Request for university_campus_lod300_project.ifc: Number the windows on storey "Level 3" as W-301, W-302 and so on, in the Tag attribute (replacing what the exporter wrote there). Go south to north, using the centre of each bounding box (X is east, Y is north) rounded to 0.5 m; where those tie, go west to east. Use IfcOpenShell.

First a look at what the model holds.

```python
import ifcopenshell
import ifcopenshell.util.element
import ifcopenshell.util.placement

model = ifcopenshell.open("university_campus_lod300_project.ifc")
print(model.schema)
storey = next(s for s in model.by_type("IfcBuildingStorey") if s.Name == "Level 3")
windows = [e for e in ifcopenshell.util.element.get_decomposition(storey) if e.is_a("IfcWindow")]
for e in sorted(windows, key=lambda e: e.id()):
    origin = ifcopenshell.util.placement.get_local_placement(e.ObjectPlacement)[:3, 3]
    print(e.id(), e.Tag, e.Name, origin.round(2) + 0.0, sep=" | ")
```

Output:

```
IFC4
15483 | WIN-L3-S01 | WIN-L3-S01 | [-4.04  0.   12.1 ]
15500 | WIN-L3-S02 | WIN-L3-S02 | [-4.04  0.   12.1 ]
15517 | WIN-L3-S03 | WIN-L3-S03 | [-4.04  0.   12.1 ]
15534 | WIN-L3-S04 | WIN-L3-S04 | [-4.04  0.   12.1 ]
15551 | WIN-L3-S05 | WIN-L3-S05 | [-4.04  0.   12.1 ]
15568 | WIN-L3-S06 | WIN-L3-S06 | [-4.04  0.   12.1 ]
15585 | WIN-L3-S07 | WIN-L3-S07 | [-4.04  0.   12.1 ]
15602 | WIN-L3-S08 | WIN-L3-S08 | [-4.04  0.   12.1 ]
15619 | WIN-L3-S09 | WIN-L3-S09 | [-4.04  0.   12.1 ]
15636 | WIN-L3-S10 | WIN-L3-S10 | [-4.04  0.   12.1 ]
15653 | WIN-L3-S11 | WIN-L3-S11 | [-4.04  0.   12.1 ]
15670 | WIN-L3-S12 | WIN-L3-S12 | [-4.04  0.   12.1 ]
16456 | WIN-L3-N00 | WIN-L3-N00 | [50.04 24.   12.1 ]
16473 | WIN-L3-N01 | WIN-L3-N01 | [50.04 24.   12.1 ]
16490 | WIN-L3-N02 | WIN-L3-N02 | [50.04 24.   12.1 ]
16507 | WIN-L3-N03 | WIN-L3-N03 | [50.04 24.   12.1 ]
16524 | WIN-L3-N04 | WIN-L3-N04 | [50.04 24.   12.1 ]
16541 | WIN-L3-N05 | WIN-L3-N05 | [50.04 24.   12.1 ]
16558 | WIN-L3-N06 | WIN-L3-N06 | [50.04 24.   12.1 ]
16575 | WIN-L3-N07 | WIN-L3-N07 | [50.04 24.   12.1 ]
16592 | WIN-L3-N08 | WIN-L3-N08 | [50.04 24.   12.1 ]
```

```python
import ifcopenshell
import ifcopenshell.geom
import ifcopenshell.util.element
import ifcopenshell.util.shape

model = ifcopenshell.open("university_campus_lod300_project.ifc")
settings = ifcopenshell.geom.settings()
settings.set("use-world-coords", True)


def centre(element):
    shape = ifcopenshell.geom.create_shape(settings, element)
    return ifcopenshell.util.shape.get_bbox_centroid(shape.geometry)


storey = next(s for s in model.by_type("IfcBuildingStorey") if s.Name == "Level 3")
windows = [e for e in ifcopenshell.util.element.get_decomposition(storey) if e.is_a("IfcWindow")]

# Insertion points can sit at a corner or the storey origin, so sort by the geometry (in metres).
centres = {e: centre(e) for e in windows}
windows.sort(key=lambda e: (round(centres[e][1] / 0.5), centres[e][0]))

for i, e in enumerate(windows, start=1):
    number = f"W-3{i:02d}"
    e.Tag = number
    print(e.id(), number)

model.write("university_campus_lod300_project_updated.ifc")
```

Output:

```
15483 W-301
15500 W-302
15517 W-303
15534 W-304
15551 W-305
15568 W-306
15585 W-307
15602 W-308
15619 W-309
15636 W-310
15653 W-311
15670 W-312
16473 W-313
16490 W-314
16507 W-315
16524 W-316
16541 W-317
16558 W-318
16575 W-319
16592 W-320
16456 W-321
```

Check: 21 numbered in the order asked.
